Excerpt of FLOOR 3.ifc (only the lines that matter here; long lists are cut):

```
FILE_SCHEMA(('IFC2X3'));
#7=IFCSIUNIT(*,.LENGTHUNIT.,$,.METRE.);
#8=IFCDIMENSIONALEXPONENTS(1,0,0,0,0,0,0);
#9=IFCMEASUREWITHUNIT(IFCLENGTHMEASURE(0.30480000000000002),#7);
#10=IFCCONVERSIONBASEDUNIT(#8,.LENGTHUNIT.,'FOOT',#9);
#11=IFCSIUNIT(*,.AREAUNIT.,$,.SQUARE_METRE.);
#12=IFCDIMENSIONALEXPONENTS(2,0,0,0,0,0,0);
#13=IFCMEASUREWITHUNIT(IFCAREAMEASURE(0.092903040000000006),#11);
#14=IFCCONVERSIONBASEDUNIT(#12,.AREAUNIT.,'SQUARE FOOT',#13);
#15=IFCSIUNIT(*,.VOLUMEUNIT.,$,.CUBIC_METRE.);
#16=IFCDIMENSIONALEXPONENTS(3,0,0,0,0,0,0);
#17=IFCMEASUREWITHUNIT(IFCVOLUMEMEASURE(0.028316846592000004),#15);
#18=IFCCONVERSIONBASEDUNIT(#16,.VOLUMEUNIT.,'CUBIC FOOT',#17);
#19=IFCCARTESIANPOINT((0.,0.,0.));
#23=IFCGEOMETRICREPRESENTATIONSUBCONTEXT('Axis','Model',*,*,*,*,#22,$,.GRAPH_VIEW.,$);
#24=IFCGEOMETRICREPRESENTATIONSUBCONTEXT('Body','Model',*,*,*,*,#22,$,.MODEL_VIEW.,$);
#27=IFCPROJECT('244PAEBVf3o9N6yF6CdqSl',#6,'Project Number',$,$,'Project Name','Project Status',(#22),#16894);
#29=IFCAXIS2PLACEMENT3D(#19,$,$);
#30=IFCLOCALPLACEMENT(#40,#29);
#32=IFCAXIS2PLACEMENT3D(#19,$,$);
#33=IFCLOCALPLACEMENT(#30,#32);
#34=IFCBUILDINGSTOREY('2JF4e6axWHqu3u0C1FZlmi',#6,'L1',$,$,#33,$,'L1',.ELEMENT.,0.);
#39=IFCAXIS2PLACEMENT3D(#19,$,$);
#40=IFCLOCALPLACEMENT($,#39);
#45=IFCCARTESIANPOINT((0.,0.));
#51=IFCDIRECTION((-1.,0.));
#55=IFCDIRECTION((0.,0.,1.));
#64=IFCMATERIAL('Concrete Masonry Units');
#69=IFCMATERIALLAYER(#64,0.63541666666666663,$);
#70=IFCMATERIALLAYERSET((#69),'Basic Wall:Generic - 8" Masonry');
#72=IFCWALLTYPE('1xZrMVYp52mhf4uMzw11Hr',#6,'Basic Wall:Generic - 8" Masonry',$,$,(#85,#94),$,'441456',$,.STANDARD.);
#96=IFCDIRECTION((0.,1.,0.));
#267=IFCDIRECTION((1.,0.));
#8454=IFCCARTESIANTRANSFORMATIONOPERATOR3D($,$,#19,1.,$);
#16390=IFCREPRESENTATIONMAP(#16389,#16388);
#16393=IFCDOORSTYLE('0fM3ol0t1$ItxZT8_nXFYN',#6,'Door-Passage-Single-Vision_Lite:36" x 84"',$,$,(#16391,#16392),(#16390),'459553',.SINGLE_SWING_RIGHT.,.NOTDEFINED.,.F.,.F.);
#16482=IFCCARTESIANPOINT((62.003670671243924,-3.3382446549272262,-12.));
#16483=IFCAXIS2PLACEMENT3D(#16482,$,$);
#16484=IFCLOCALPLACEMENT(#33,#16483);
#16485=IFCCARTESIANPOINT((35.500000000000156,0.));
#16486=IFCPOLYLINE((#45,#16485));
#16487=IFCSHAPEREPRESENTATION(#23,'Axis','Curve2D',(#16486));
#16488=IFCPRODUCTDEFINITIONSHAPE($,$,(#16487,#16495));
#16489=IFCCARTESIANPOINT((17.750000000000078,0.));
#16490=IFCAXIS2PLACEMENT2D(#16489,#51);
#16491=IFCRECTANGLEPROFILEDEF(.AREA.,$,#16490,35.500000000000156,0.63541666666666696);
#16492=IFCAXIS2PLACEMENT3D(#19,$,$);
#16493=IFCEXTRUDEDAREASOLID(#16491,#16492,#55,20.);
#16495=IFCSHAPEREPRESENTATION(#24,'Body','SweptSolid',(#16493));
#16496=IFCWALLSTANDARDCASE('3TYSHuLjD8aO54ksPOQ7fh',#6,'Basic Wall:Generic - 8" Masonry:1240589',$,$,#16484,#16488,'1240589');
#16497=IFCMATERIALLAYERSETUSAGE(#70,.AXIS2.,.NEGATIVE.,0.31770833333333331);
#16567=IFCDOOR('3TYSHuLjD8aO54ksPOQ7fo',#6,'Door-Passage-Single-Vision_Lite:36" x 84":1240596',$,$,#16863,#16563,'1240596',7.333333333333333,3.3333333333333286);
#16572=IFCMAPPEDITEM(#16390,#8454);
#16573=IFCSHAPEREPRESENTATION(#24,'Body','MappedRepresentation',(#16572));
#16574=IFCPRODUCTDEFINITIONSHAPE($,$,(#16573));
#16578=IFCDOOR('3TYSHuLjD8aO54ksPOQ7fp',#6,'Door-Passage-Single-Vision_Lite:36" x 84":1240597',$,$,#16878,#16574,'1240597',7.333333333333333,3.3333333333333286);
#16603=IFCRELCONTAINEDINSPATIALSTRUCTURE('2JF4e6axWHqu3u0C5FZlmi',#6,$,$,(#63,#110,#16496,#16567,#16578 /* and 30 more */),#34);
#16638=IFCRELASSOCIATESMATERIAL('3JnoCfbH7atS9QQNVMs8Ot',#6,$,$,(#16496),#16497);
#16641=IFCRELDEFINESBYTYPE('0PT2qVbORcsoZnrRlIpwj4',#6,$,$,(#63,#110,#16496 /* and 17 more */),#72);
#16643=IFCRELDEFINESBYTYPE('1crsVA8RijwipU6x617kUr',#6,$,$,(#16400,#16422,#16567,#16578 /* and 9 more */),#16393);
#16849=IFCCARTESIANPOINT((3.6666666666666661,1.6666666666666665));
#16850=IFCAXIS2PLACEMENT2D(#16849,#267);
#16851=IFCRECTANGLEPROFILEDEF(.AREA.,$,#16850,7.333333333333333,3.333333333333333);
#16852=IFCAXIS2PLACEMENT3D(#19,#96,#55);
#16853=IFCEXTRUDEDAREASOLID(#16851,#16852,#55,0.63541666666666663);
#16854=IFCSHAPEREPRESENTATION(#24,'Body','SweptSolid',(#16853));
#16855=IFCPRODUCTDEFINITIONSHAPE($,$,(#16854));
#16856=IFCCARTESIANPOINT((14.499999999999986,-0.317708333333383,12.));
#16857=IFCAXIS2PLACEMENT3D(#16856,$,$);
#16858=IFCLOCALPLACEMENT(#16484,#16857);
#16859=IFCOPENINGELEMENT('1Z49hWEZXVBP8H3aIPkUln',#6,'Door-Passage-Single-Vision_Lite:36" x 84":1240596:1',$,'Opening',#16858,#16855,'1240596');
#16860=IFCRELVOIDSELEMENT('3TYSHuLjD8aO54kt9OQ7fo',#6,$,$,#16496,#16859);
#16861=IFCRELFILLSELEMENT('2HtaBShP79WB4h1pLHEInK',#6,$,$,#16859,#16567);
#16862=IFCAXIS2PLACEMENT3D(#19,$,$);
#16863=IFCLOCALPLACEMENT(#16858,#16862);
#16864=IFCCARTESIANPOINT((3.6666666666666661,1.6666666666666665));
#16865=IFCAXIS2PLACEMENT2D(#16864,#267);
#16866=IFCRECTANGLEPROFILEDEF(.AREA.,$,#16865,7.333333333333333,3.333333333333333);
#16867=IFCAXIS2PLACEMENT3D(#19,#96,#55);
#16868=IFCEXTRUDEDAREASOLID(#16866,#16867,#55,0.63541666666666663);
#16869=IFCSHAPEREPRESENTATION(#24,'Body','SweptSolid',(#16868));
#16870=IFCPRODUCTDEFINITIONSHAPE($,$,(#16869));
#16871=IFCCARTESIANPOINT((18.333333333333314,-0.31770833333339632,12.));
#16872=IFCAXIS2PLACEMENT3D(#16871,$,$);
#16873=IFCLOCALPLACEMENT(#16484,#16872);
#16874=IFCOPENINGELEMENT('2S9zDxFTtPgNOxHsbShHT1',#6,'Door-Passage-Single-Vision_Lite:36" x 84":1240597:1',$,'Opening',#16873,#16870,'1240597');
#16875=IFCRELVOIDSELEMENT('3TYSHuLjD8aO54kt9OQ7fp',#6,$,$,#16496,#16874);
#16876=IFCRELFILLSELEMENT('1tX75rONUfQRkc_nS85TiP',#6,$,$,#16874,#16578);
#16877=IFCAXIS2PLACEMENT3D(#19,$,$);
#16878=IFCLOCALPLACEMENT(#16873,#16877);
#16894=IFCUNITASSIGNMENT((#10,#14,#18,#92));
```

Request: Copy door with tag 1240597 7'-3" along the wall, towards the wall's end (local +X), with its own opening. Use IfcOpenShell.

```python
import ifcopenshell
import ifcopenshell.api.feature
import ifcopenshell.api.geometry
import ifcopenshell.api.root
import ifcopenshell.geom
import ifcopenshell.util.element
import ifcopenshell.util.placement
import ifcopenshell.util.shape
import ifcopenshell.util.unit

model = ifcopenshell.open("FLOOR 3.ifc")
unit_scale = ifcopenshell.util.unit.calculate_unit_scale(model)
settings = ifcopenshell.geom.settings()


def volume(element):
    """Net volume in cubic metres, openings subtracted."""
    shape = ifcopenshell.geom.create_shape(settings, element)
    return ifcopenshell.util.shape.get_volume(shape.geometry)


def reuse_history(source, copy):
    """copy_class also copies each property set's owner history, people and application; keep the originals."""
    for rel in copy.IsDefinedBy:
        if rel.is_a("IfcRelDefinesByProperties") and (history := rel.RelatingPropertyDefinition.OwnerHistory):
            rel.RelatingPropertyDefinition.OwnerHistory = source.OwnerHistory
            ifcopenshell.util.element.remove_deep2(model, history)


door = model.by_guid("3TYSHuLjD8aO54ksPOQ7fp")
opening = door.FillsVoids[0].RelatingOpeningElement
wall = opening.VoidsElements[0].RelatingBuildingElement
before = volume(wall)
shift = ifcopenshell.util.placement.get_local_placement(wall.ObjectPlacement)[:3, 0] * 87 * 0.0254 / unit_scale

# copy_class copies the void relationship, type, container and properties, but no geometry.
new_opening = ifcopenshell.api.root.copy_class(model, product=opening)
new_opening.Representation = ifcopenshell.util.element.copy_deep(
    model, opening.Representation, exclude=["IfcGeometricRepresentationContext", "IfcRepresentationMap"]
)
new_opening.Name = 'Door-Passage-Single-Vision_Lite:36" x 84"'
new_opening.Tag = None
new_door = ifcopenshell.api.root.copy_class(model, product=door)
new_door.Representation = ifcopenshell.util.element.copy_deep(
    model, door.Representation, exclude=["IfcGeometricRepresentationContext", "IfcRepresentationMap"]
)
new_door.Name = 'Door-Passage-Single-Vision_Lite:36" x 84"'
new_door.Tag = None
reuse_history(door, new_door)
fills = ifcopenshell.api.feature.add_filling(model, opening=new_opening, element=new_door)
fills.OwnerHistory = new_door.OwnerHistory  # required in IFC2X3

for old, new in ((opening, new_opening), (door, new_door)):
    matrix = ifcopenshell.util.placement.get_local_placement(old.ObjectPlacement)
    matrix[:3, 3] += shift
    ifcopenshell.api.geometry.edit_object_placement(model, product=new, matrix=matrix, is_si=False)

after = volume(wall)

print(f"wall volume {before:.3f} -> {after:.3f} m3")

model.write("FLOOR 3_updated.ifc")
```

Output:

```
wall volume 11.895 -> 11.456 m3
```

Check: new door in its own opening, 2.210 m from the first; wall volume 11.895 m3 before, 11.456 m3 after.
